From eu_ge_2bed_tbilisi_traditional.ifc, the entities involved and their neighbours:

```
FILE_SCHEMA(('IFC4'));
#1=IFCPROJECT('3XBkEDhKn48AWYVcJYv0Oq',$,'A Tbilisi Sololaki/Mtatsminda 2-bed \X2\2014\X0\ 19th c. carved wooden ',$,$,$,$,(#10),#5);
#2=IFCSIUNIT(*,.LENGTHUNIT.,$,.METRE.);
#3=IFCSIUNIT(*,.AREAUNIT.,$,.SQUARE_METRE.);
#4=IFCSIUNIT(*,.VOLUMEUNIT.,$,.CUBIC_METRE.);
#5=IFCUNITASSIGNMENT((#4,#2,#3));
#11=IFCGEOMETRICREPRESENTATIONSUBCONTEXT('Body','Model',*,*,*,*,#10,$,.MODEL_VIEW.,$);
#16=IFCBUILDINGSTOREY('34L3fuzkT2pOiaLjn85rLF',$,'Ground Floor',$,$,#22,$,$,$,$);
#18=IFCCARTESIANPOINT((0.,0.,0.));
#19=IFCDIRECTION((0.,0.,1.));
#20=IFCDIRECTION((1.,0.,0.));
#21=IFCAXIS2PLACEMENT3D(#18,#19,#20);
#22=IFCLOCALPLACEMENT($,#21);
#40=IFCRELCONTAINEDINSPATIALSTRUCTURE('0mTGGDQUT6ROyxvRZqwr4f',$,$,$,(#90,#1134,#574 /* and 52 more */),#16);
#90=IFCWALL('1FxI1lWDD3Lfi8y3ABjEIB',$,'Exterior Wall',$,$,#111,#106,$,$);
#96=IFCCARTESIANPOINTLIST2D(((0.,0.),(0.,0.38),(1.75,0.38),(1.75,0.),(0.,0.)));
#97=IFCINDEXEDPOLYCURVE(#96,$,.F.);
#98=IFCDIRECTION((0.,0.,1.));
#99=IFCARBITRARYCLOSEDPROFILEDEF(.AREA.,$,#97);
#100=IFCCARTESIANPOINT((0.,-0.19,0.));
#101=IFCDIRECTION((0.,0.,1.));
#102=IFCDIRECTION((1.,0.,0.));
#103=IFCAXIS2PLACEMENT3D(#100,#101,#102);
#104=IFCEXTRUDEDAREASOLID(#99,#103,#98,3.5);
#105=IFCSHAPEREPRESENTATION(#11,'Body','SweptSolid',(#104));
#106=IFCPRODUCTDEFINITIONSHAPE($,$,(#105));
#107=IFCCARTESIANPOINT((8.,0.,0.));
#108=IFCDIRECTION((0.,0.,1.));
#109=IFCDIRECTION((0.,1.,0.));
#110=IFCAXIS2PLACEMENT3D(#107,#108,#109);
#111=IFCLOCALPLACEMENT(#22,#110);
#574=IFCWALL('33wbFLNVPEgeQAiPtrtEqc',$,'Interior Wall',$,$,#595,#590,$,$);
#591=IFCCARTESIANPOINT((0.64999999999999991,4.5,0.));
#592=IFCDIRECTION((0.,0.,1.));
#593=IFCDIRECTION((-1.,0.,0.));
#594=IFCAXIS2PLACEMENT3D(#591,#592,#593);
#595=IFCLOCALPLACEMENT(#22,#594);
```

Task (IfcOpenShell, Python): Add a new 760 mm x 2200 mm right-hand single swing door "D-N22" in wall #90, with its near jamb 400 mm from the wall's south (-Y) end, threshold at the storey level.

```python
import numpy as np
import ifcopenshell
import ifcopenshell.api.feature
import ifcopenshell.api.geometry
import ifcopenshell.api.root
import ifcopenshell.api.spatial
import ifcopenshell.geom
import ifcopenshell.util.element
import ifcopenshell.util.placement
import ifcopenshell.util.representation
import ifcopenshell.util.shape
import ifcopenshell.util.unit

model = ifcopenshell.open("eu_ge_2bed_tbilisi_traditional.ifc")
unit_scale = ifcopenshell.util.unit.calculate_unit_scale(model)
settings = ifcopenshell.geom.settings()


def volume(element):
    """Net volume in cubic metres, openings subtracted."""
    shape = ifcopenshell.geom.create_shape(settings, element)
    return ifcopenshell.util.shape.get_volume(shape.geometry)


wall = model.by_guid("1FxI1lWDD3Lfi8y3ABjEIB")
storey = ifcopenshell.util.element.get_container(wall, ifc_class="IfcBuildingStorey")
context = ifcopenshell.util.representation.get_context(model, "Model", "Body", "MODEL_VIEW")
before = volume(wall)

width, height, from_end, sill = 0.76, 2.2, 0.4, 0.0  # metres

# The wall runs along its own X axis, and the end named is its -X end.
wall_shape = ifcopenshell.geom.create_shape(settings, wall)
x, y, z = ifcopenshell.util.shape.get_vertices(wall_shape.geometry).T
start = x.min() + from_end
face, thickness = float(y.min()), float(y.max() - y.min())
wall_matrix = ifcopenshell.util.placement.get_local_placement(wall.ObjectPlacement)
level = ifcopenshell.util.placement.get_local_placement(storey.ObjectPlacement)[2, 3]


def in_wall(x, y):
    """Placement at x, y metres in the wall's axes, at sill height."""
    matrix = wall_matrix.copy()
    matrix[:, 3] = wall_matrix @ np.array([x / unit_scale, y / unit_scale, 0.0, 1.0])
    matrix[2, 3] = level + sill / unit_scale
    return matrix


# Opening: a box that overshoots both wall faces by 50 mm.
opening = ifcopenshell.api.root.create_entity(model, ifc_class="IfcOpeningElement", predefined_type="OPENING")
box = ifcopenshell.api.geometry.add_wall_representation(
    model, context=context, length=width, height=height, thickness=thickness + 0.1
)
ifcopenshell.api.geometry.assign_representation(model, product=opening, representation=box)
ifcopenshell.api.geometry.edit_object_placement(model, product=opening, matrix=in_wall(start, face - 0.05), is_si=False)
ifcopenshell.api.feature.add_feature(model, feature=opening, element=wall)

door = ifcopenshell.api.root.create_entity(model, ifc_class="IfcDoor", name="D-N22", predefined_type="DOOR")
door.OverallWidth, door.OverallHeight = width / unit_scale, height / unit_scale
door.OperationType = "SINGLE_SWING_RIGHT"
body = ifcopenshell.api.geometry.add_door_representation(
    model,
    context=context,
    overall_width=door.OverallWidth,
    overall_height=door.OverallHeight,
    operation_type="SINGLE_SWING_RIGHT",
    lining_properties={"LiningDepth": thickness / unit_scale, "ThresholdDepth": thickness / unit_scale},
)
ifcopenshell.api.geometry.assign_representation(model, product=door, representation=body)
ifcopenshell.api.spatial.assign_container(model, products=[door], relating_structure=storey)
ifcopenshell.api.feature.add_filling(model, opening=opening, element=door)

# The lining spans the wall, so the door starts at the wall face.
ifcopenshell.api.geometry.edit_object_placement(model, product=door, matrix=in_wall(start, face), is_si=False)

after = volume(wall)

print(f"wall volume {before:.3f} -> {after:.3f} m3")

model.write("eu_ge_2bed_tbilisi_traditional-out.ifc")
```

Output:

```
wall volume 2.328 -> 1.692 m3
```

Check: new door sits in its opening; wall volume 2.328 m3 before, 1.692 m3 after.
